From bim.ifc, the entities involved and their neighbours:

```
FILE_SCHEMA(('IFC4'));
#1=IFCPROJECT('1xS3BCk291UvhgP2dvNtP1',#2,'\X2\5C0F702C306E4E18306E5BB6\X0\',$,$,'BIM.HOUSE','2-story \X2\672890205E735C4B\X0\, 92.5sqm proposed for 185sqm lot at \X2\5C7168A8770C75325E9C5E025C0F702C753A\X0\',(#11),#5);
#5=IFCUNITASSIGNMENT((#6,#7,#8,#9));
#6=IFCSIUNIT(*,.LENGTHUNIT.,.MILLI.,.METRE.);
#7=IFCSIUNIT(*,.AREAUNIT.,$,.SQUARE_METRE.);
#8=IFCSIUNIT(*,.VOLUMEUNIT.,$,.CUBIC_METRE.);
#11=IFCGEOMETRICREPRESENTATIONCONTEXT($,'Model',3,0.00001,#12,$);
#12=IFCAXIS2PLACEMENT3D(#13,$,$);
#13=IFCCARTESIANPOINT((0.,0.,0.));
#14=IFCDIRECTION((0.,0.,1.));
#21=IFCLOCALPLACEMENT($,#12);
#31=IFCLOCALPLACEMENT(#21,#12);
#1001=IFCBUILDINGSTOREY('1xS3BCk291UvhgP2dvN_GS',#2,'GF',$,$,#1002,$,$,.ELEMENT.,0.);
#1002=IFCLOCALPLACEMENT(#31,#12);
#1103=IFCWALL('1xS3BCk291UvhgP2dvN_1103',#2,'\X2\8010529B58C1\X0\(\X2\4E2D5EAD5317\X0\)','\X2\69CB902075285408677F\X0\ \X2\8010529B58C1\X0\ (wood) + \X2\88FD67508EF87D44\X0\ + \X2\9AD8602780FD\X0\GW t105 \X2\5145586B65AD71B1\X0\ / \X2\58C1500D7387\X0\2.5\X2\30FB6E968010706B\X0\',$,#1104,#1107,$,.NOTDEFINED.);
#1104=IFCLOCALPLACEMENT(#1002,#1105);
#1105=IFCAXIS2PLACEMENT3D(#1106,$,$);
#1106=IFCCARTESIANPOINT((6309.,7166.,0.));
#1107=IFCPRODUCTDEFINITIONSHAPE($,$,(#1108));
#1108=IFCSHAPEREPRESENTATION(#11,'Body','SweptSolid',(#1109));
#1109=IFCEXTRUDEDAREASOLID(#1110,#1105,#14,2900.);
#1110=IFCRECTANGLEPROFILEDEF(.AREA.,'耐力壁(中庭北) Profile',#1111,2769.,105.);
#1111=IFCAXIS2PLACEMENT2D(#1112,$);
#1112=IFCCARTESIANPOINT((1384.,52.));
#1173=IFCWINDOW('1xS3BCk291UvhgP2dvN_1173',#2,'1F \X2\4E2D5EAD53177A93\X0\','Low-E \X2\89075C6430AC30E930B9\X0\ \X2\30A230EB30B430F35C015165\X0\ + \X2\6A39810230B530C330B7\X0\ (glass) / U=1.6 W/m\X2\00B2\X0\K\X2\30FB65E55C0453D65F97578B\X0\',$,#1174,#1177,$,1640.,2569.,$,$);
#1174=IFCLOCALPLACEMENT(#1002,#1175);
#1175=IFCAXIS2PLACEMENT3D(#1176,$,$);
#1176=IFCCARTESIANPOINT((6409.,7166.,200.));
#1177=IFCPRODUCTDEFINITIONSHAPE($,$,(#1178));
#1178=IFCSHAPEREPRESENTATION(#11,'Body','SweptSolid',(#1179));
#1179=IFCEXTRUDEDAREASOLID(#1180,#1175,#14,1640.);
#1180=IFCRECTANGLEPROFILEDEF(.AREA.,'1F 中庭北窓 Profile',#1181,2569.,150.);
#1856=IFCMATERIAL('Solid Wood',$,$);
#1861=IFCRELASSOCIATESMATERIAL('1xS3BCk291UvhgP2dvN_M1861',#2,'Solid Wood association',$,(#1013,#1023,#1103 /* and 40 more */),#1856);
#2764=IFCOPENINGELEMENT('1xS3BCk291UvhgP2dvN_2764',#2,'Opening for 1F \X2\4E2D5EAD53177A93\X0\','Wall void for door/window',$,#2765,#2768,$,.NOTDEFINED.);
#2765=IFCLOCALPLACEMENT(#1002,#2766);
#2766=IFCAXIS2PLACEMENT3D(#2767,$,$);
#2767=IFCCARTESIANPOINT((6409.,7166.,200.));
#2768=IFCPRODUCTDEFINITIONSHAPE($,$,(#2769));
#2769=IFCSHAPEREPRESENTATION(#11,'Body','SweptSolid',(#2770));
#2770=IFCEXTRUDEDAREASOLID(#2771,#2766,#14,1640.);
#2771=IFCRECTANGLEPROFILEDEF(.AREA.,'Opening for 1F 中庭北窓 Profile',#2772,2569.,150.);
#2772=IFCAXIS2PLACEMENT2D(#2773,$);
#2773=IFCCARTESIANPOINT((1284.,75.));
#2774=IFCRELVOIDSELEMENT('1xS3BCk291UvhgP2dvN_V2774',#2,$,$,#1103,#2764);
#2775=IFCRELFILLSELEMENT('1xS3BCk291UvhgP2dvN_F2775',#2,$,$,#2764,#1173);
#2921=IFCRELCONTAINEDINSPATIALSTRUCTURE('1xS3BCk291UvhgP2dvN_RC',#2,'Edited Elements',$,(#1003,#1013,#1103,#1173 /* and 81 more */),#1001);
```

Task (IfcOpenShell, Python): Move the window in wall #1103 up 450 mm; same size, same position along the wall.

```python
import numpy as np
import ifcopenshell
import ifcopenshell.api.geometry
import ifcopenshell.util.placement
import ifcopenshell.util.unit

model = ifcopenshell.open("bim.ifc")
unit_scale = ifcopenshell.util.unit.calculate_unit_scale(model)

window = model.by_guid("1xS3BCk291UvhgP2dvN_1173")
opening = window.FillsVoids[0].RelatingOpeningElement
dz = 0.45 / unit_scale

shift = np.array([0.0, 0.0, dz])
# The window is not placed relative to its opening, so move both.
for product in (opening, window):
    matrix = ifcopenshell.util.placement.get_local_placement(product.ObjectPlacement)
    matrix[:3, 3] += shift
    ifcopenshell.api.geometry.edit_object_placement(model, product=product, matrix=matrix, is_si=False)

print(f"moved by {dz * unit_scale:+.3f} m")

model.write("bim_edited.ifc")
```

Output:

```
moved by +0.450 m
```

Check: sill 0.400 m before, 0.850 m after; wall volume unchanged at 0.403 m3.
